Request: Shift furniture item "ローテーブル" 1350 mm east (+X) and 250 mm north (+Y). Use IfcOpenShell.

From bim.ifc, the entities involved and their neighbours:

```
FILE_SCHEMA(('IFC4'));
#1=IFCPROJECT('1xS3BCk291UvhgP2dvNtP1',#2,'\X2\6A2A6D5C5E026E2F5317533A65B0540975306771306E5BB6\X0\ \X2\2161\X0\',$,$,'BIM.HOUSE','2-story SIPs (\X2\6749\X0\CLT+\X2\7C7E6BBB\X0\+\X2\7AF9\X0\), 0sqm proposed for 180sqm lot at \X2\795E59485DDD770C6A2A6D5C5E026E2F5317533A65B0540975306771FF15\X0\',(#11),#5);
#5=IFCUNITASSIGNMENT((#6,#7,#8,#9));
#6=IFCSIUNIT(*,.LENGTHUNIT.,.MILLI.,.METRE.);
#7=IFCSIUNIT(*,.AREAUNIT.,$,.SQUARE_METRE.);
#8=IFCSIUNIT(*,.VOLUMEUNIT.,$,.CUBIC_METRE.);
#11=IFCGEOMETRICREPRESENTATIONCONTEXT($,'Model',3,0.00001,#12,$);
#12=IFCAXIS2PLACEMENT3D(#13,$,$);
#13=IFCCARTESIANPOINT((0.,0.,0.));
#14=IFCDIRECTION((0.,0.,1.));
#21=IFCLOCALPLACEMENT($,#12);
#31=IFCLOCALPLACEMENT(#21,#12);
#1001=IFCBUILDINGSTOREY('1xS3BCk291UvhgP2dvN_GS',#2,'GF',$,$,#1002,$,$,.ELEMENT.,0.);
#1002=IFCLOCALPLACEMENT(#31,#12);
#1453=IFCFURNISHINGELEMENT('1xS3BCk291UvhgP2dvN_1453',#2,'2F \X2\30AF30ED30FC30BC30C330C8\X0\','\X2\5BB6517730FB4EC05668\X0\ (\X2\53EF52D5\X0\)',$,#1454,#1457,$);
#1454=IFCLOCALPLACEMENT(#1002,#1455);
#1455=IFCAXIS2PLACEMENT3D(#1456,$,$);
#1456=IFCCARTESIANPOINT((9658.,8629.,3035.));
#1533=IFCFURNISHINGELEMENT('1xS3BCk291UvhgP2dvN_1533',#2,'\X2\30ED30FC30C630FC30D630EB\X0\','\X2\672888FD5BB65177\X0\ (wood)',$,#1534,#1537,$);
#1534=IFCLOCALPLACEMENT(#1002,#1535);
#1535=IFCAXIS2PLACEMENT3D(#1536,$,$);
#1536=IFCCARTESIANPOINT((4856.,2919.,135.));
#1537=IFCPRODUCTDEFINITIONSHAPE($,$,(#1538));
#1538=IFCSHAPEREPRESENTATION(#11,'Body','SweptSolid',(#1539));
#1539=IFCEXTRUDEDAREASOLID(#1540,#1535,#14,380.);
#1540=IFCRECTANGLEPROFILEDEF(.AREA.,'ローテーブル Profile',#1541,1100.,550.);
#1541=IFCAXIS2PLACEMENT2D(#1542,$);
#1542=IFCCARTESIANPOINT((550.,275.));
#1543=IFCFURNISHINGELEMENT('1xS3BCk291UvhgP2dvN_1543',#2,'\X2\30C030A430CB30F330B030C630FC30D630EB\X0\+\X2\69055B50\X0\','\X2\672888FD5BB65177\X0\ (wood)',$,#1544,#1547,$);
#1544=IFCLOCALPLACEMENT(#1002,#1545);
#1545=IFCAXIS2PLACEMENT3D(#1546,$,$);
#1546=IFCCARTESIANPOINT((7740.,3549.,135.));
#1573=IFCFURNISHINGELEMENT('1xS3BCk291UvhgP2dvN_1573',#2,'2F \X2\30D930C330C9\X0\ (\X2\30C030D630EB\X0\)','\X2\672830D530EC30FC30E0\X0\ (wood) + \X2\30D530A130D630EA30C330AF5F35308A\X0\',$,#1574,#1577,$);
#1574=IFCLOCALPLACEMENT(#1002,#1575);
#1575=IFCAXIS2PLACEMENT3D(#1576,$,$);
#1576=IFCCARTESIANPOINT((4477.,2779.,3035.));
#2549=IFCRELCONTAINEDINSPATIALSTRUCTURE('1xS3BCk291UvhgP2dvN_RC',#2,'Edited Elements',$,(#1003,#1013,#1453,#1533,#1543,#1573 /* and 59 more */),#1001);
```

```python
import ifcopenshell
import ifcopenshell.api.geometry
import ifcopenshell.util.placement
import ifcopenshell.util.unit

model = ifcopenshell.open("bim.ifc")
unit_scale = ifcopenshell.util.unit.calculate_unit_scale(model)

item = model.by_guid("1xS3BCk291UvhgP2dvN_1533")
matrix = ifcopenshell.util.placement.get_local_placement(item.ObjectPlacement)
matrix[0, 3] += 1.35 / unit_scale
matrix[1, 3] += 0.25 / unit_scale
ifcopenshell.api.geometry.edit_object_placement(model, product=item, matrix=matrix, is_si=False)

print(ifcopenshell.util.placement.get_local_placement(item.ObjectPlacement).round(3) + 0.0)

model.write("bim_v2.ifc")
```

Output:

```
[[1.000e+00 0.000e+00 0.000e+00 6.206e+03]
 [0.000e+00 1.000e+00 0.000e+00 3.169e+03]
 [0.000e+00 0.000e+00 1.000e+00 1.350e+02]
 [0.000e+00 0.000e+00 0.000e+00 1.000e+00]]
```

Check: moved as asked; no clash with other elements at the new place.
